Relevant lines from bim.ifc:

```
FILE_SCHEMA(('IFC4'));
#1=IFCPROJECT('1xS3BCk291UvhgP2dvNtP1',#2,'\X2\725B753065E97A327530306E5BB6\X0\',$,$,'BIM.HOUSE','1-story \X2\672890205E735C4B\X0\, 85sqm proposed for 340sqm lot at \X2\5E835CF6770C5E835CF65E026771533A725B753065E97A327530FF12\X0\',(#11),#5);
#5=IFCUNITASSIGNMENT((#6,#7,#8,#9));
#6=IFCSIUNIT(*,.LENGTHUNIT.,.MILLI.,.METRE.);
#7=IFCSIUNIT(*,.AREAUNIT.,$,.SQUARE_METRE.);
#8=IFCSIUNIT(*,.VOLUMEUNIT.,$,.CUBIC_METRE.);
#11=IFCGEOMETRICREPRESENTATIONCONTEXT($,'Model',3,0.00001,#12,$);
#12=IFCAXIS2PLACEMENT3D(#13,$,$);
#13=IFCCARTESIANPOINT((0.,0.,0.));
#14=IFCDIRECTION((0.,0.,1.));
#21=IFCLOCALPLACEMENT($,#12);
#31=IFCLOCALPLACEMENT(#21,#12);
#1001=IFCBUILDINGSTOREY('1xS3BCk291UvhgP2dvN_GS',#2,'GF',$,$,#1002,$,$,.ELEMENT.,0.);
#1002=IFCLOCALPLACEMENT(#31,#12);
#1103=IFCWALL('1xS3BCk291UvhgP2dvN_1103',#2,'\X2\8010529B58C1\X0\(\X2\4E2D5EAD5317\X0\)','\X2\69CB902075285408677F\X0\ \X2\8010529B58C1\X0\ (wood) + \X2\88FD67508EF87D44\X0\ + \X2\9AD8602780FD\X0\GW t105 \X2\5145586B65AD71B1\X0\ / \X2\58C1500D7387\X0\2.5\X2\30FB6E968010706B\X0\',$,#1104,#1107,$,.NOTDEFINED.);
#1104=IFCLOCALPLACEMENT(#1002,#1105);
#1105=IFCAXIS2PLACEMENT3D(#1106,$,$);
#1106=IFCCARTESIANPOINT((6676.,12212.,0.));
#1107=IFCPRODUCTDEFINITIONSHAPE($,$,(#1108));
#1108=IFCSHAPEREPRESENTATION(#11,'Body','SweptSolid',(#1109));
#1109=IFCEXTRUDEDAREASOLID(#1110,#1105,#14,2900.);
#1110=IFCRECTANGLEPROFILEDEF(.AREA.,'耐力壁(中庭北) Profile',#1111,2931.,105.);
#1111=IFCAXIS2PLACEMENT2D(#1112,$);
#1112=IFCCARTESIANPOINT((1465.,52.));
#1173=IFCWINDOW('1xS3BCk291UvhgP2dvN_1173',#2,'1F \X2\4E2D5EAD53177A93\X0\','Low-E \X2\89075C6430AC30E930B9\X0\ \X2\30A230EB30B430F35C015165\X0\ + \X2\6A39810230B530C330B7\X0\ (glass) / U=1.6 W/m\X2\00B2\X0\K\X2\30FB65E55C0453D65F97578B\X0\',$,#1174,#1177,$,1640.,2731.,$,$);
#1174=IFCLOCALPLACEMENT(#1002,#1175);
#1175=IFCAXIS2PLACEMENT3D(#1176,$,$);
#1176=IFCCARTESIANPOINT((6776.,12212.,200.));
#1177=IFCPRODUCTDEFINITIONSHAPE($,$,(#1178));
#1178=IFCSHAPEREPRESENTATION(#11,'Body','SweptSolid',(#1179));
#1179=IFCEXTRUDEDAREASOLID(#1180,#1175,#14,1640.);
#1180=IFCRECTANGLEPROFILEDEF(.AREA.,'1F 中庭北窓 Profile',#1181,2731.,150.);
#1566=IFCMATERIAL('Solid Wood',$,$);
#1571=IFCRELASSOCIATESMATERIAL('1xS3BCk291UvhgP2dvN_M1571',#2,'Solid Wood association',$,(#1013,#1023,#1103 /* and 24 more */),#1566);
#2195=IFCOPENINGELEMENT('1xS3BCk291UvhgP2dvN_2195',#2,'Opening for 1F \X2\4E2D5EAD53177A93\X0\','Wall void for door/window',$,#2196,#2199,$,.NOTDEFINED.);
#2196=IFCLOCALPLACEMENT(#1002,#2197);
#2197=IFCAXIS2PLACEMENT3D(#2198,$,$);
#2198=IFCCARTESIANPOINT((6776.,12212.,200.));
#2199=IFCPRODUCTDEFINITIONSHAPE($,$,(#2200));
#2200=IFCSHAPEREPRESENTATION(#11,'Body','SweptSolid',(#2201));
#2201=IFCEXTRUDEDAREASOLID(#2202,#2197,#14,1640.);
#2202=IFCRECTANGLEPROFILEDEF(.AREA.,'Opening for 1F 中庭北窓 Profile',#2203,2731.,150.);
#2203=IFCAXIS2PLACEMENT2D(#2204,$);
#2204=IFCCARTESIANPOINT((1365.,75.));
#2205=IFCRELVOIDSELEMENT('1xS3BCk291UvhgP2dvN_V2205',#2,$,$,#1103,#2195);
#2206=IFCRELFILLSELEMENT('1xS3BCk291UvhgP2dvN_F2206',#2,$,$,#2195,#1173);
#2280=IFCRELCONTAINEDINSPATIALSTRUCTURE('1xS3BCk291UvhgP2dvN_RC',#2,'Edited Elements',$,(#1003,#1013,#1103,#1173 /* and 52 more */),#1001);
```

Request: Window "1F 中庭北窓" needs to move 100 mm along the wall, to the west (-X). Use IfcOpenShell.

```python
import ifcopenshell
import ifcopenshell.api.geometry
import ifcopenshell.util.placement
import ifcopenshell.util.unit

model = ifcopenshell.open("bim.ifc")
unit_scale = ifcopenshell.util.unit.calculate_unit_scale(model)

window = model.by_guid("1xS3BCk291UvhgP2dvN_1173")
opening = window.FillsVoids[0].RelatingOpeningElement
wall = opening.VoidsElements[0].RelatingBuildingElement

wall_matrix = ifcopenshell.util.placement.get_local_placement(wall.ObjectPlacement)
shift = wall_matrix[:3, 0] * -0.1 / unit_scale
before = ifcopenshell.util.placement.get_local_placement(window.ObjectPlacement)[:3, 3].copy()

# The window is not placed relative to its opening, so move both.
for product in (opening, window):
    matrix = ifcopenshell.util.placement.get_local_placement(product.ObjectPlacement)
    matrix[:3, 3] += shift
    ifcopenshell.api.geometry.edit_object_placement(model, product=product, matrix=matrix, is_si=False)

after = ifcopenshell.util.placement.get_local_placement(window.ObjectPlacement)[:3, 3]
print("window moved by", (after - before).round(3) + 0.0)

model.write("bim-out.ifc")
```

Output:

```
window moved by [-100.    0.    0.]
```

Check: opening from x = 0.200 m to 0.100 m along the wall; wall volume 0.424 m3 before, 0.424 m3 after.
